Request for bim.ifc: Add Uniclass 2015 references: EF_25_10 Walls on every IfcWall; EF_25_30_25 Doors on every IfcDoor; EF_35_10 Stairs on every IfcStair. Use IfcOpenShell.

First a look at what the model holds.

```python
import ifcopenshell

model = ifcopenshell.open("bim.ifc")
print(model.schema)
print("classifications:", [c.Name for c in model.by_type("IfcClassification")])
for ifc_class in ("IfcDoor", "IfcRoof", "IfcStair", "IfcWall", "IfcWindow"):
    print(ifc_class, len(model.by_type(ifc_class)))
```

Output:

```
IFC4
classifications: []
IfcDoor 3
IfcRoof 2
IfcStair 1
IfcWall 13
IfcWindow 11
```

```python
import ifcopenshell
import ifcopenshell.api.classification

model = ifcopenshell.open("bim.ifc")

system = ifcopenshell.api.classification.add_classification(model, classification="Uniclass 2015")

codes = {
    "IfcWall": ("EF_25_10", "Walls"),
    "IfcDoor": ("EF_25_30_25", "Doors"),
    "IfcStair": ("EF_35_10", "Stairs"),
}
for ifc_class, (code, name) in codes.items():
    products = model.by_type(ifc_class)
    ifcopenshell.api.classification.add_reference(
        model, products=products, classification=system, identification=code, name=name
    )
    print(code, len(products))

model.write("bim_updated.ifc")
```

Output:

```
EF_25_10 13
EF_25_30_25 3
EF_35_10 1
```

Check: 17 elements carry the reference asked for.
